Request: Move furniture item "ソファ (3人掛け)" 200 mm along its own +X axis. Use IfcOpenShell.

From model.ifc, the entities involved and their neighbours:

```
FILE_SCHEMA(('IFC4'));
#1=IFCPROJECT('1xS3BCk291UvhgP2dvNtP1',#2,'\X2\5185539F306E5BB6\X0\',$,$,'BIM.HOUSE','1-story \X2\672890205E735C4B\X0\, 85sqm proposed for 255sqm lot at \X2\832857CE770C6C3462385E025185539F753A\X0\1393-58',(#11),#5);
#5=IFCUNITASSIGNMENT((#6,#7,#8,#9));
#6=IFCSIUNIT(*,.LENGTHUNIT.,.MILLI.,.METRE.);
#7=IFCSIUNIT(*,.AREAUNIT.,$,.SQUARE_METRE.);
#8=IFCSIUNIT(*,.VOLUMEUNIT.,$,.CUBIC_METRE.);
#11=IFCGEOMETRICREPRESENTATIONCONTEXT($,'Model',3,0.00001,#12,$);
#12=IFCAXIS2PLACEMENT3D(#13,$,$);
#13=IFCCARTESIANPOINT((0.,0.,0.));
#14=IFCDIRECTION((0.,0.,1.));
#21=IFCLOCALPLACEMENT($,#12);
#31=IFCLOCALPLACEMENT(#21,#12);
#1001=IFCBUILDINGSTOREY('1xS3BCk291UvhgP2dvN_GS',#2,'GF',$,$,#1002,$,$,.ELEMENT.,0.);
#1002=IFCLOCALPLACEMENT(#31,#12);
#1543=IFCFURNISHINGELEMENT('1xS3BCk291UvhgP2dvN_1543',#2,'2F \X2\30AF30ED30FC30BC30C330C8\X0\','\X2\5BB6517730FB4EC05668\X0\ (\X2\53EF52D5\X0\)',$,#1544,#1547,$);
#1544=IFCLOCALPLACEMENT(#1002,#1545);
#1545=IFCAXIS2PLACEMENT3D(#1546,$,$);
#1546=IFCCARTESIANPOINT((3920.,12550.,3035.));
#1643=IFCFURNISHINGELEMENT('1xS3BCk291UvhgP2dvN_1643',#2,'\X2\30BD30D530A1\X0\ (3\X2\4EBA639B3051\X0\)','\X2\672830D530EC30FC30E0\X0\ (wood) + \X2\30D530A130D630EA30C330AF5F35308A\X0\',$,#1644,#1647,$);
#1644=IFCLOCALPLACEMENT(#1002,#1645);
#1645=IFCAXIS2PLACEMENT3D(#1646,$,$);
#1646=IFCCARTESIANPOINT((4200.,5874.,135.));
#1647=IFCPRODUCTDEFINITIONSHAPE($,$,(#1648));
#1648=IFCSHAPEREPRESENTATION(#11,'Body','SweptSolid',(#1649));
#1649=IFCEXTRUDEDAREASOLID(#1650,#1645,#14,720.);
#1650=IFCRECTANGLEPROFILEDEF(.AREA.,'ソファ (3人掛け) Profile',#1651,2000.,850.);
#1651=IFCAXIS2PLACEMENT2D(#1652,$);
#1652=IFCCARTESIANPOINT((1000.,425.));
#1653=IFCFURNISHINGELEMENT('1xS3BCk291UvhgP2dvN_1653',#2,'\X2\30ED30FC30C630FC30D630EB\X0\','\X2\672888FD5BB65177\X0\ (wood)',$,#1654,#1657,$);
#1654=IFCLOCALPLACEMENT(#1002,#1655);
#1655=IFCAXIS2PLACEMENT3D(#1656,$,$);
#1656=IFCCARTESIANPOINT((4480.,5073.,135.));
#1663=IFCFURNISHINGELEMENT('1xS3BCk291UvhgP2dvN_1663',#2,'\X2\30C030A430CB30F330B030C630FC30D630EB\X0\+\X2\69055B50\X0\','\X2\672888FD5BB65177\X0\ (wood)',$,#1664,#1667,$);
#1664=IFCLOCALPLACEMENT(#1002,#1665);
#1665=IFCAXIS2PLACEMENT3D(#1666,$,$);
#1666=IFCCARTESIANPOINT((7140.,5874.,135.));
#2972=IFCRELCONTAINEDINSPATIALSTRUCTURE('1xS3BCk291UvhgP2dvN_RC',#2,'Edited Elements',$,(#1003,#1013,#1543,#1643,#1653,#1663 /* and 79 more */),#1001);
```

```python
import ifcopenshell
import ifcopenshell.api.geometry
import ifcopenshell.util.placement
import ifcopenshell.util.unit

model = ifcopenshell.open("model.ifc")
unit_scale = ifcopenshell.util.unit.calculate_unit_scale(model)

item = model.by_guid("1xS3BCk291UvhgP2dvN_1643")
matrix = ifcopenshell.util.placement.get_local_placement(item.ObjectPlacement)
matrix[:3, 3] += matrix[:3, 0] * 0.2 / unit_scale
ifcopenshell.api.geometry.edit_object_placement(model, product=item, matrix=matrix, is_si=False)

print(ifcopenshell.util.placement.get_local_placement(item.ObjectPlacement).round(3) + 0.0)

model.write("model_edited.ifc")
```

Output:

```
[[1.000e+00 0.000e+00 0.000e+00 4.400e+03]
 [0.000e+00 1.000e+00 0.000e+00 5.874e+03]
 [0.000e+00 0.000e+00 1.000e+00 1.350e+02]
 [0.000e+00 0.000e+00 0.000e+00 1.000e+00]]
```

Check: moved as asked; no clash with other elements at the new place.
